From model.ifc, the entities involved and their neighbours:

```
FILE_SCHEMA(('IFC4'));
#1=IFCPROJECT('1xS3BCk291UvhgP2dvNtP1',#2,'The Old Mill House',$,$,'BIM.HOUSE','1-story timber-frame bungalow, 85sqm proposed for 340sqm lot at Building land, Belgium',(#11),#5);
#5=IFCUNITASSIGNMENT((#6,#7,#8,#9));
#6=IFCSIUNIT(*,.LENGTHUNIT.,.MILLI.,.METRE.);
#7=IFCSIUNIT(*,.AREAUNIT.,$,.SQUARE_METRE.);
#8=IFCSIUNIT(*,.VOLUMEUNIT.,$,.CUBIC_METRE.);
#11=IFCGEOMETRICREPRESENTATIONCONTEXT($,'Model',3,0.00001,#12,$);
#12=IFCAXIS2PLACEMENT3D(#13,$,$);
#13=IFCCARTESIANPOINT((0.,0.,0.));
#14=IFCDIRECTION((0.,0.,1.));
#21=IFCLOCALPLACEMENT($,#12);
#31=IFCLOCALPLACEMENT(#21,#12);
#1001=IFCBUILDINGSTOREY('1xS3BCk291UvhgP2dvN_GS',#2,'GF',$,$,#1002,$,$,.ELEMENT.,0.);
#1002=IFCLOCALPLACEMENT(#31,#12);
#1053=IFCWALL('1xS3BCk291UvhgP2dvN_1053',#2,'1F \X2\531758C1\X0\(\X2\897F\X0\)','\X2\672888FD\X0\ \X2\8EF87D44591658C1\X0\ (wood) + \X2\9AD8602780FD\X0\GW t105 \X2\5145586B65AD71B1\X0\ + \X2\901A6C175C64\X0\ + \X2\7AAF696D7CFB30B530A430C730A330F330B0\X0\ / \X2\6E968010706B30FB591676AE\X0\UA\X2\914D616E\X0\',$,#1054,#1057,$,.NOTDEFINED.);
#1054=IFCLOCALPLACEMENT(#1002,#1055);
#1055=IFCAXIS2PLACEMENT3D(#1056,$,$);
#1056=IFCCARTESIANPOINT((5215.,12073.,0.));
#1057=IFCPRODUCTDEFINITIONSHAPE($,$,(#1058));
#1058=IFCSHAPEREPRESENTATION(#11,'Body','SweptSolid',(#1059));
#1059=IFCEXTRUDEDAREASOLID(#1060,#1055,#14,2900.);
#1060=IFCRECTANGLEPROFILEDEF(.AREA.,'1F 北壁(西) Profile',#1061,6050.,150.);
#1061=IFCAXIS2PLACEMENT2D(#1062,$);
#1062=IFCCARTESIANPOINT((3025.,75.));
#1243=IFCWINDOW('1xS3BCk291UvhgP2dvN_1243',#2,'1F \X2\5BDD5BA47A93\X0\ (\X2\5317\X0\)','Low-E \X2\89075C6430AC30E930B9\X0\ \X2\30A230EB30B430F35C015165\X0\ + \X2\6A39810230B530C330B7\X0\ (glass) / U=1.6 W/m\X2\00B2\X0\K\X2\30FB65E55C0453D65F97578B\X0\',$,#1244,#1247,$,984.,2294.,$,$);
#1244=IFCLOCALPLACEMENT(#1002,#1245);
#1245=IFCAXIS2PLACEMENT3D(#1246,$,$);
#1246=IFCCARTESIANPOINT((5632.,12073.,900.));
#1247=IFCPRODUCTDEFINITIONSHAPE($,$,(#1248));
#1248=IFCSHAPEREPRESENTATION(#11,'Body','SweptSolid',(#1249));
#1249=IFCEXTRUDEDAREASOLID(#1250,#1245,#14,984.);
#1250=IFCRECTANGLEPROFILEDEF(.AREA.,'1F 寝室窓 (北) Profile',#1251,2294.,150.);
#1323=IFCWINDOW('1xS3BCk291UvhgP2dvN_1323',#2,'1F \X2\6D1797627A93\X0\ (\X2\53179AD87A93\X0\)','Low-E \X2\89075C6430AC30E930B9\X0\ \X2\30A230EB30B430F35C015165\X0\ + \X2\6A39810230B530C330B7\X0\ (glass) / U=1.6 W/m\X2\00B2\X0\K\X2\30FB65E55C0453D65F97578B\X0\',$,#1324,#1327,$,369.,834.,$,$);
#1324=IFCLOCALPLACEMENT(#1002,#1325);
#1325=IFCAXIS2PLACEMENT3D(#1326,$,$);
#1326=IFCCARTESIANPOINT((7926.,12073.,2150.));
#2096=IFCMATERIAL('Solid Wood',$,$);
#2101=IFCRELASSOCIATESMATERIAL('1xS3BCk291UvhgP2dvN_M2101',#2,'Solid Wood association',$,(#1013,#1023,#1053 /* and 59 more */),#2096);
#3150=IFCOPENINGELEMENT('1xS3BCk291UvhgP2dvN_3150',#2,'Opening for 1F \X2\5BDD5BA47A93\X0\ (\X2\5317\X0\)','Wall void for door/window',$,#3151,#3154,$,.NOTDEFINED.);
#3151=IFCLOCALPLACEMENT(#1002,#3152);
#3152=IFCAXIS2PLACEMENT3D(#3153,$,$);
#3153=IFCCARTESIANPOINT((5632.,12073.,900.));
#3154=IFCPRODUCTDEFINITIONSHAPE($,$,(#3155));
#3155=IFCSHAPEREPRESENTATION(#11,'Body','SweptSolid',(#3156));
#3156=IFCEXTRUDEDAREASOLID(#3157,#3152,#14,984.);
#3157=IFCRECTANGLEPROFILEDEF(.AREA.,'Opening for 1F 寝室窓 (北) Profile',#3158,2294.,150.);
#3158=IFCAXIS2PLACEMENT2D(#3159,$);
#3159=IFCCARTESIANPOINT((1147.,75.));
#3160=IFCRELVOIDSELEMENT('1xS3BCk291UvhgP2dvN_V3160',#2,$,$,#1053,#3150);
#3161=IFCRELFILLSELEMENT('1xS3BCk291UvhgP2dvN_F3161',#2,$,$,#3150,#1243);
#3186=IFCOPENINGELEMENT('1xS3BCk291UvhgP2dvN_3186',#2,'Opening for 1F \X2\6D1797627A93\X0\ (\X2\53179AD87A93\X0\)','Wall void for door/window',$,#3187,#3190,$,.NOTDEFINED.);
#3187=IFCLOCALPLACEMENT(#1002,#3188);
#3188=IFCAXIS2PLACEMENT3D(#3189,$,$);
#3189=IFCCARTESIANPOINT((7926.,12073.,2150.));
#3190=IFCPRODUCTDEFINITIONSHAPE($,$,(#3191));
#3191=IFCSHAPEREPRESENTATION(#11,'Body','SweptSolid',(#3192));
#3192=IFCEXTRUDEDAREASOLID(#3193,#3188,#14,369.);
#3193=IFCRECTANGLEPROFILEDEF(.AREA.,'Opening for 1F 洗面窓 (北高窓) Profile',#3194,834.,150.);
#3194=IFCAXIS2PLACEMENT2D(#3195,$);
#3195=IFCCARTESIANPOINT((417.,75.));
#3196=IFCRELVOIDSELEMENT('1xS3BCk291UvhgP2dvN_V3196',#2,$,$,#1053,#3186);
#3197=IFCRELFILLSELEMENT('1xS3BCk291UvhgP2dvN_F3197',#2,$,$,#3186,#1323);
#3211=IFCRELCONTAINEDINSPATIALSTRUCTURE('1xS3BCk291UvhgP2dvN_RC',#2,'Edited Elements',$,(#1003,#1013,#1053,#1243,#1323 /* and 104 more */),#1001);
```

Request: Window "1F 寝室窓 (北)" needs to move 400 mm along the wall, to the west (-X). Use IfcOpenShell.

```python
import ifcopenshell
import ifcopenshell.api.geometry
import ifcopenshell.util.placement
import ifcopenshell.util.unit

model = ifcopenshell.open("model.ifc")
unit_scale = ifcopenshell.util.unit.calculate_unit_scale(model)

window = model.by_guid("1xS3BCk291UvhgP2dvN_1243")
opening = window.FillsVoids[0].RelatingOpeningElement
wall = opening.VoidsElements[0].RelatingBuildingElement

wall_matrix = ifcopenshell.util.placement.get_local_placement(wall.ObjectPlacement)
shift = wall_matrix[:3, 0] * -0.4 / unit_scale
before = ifcopenshell.util.placement.get_local_placement(window.ObjectPlacement)[:3, 3].copy()

# The window is not placed relative to its opening, so move both.
for product in (opening, window):
    matrix = ifcopenshell.util.placement.get_local_placement(product.ObjectPlacement)
    matrix[:3, 3] += shift
    ifcopenshell.api.geometry.edit_object_placement(model, product=product, matrix=matrix, is_si=False)

after = ifcopenshell.util.placement.get_local_placement(window.ObjectPlacement)[:3, 3]
print("window moved by", (after - before).round(3) + 0.0)

model.write("model_v2.ifc")
```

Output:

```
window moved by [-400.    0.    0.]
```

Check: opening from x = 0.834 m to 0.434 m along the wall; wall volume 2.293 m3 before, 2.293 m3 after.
